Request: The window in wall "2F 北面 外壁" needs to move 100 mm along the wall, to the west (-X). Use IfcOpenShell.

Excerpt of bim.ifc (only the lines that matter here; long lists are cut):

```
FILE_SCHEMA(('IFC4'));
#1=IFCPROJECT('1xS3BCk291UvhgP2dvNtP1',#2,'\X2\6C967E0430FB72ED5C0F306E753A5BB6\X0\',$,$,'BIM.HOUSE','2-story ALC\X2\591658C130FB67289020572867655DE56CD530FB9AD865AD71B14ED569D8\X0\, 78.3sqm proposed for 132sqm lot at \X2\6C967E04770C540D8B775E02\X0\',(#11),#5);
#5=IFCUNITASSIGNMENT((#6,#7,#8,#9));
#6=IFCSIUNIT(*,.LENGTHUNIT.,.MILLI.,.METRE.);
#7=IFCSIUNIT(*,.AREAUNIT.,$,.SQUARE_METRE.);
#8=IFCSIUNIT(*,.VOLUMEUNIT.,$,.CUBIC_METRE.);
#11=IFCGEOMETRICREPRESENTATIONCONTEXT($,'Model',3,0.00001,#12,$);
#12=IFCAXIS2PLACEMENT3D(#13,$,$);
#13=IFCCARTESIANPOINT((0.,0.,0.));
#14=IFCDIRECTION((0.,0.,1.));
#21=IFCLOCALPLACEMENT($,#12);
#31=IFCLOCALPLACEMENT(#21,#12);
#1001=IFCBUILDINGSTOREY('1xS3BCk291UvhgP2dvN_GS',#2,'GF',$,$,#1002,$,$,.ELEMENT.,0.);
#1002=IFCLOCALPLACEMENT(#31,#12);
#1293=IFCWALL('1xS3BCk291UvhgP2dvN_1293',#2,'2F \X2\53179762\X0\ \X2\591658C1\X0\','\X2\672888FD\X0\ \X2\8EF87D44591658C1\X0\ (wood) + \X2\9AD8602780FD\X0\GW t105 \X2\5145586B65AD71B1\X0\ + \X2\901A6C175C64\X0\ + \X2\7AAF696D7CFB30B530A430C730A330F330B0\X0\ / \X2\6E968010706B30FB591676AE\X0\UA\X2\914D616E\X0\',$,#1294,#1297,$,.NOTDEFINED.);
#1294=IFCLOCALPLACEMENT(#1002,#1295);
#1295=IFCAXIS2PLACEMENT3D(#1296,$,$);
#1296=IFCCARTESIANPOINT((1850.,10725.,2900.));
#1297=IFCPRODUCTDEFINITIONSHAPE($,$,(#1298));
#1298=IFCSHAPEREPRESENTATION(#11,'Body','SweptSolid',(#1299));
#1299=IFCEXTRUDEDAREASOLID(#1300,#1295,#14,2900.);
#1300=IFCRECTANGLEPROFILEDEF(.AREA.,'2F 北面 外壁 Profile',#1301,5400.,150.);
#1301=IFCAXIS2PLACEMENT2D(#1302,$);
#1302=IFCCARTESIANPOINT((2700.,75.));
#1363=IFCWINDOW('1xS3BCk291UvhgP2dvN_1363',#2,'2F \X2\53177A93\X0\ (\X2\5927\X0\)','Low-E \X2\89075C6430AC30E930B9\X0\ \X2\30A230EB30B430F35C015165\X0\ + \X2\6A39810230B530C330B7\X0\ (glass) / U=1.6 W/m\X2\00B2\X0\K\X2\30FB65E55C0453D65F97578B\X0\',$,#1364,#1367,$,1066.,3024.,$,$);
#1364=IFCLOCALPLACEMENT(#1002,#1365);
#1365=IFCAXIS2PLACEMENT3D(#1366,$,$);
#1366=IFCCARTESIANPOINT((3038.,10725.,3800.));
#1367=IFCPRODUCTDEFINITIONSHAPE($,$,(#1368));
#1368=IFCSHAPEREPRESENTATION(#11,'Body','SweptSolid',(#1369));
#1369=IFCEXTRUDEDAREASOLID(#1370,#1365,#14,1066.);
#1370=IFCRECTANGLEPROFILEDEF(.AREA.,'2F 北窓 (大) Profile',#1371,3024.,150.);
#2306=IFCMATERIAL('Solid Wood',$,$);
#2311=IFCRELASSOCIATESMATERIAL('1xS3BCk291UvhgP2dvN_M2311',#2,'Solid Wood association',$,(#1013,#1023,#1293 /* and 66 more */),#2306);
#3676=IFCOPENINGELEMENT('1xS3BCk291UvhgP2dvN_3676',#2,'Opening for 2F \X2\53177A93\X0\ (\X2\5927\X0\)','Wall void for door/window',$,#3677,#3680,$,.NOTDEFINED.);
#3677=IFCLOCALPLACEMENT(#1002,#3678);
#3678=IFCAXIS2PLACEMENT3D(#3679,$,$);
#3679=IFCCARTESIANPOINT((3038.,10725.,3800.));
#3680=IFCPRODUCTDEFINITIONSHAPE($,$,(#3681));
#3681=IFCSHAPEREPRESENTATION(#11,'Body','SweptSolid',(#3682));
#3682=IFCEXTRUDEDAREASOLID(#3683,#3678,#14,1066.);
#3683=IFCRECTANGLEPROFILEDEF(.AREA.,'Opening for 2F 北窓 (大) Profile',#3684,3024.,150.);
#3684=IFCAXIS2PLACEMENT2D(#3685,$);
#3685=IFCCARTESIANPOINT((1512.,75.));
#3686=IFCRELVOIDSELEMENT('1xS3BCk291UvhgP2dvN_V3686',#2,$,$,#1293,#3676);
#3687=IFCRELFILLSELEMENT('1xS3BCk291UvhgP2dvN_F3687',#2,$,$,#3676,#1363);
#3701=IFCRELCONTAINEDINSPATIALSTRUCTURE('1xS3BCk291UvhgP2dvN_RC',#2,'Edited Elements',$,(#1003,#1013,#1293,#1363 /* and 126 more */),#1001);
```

```python
import ifcopenshell
import ifcopenshell.api.geometry
import ifcopenshell.util.placement
import ifcopenshell.util.unit

model = ifcopenshell.open("bim.ifc")
unit_scale = ifcopenshell.util.unit.calculate_unit_scale(model)

window = model.by_guid("1xS3BCk291UvhgP2dvN_1363")
opening = window.FillsVoids[0].RelatingOpeningElement
wall = opening.VoidsElements[0].RelatingBuildingElement

wall_matrix = ifcopenshell.util.placement.get_local_placement(wall.ObjectPlacement)
shift = wall_matrix[:3, 0] * -0.1 / unit_scale
before = ifcopenshell.util.placement.get_local_placement(window.ObjectPlacement)[:3, 3].copy()

# The window is not placed relative to its opening, so move both.
for product in (opening, window):
    matrix = ifcopenshell.util.placement.get_local_placement(product.ObjectPlacement)
    matrix[:3, 3] += shift
    ifcopenshell.api.geometry.edit_object_placement(model, product=product, matrix=matrix, is_si=False)

after = ifcopenshell.util.placement.get_local_placement(window.ObjectPlacement)[:3, 3]
print("window moved by", (after - before).round(3) + 0.0)

model.write("bim-out.ifc")
```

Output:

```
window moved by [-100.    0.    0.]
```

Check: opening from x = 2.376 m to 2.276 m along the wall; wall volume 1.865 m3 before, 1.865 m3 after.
